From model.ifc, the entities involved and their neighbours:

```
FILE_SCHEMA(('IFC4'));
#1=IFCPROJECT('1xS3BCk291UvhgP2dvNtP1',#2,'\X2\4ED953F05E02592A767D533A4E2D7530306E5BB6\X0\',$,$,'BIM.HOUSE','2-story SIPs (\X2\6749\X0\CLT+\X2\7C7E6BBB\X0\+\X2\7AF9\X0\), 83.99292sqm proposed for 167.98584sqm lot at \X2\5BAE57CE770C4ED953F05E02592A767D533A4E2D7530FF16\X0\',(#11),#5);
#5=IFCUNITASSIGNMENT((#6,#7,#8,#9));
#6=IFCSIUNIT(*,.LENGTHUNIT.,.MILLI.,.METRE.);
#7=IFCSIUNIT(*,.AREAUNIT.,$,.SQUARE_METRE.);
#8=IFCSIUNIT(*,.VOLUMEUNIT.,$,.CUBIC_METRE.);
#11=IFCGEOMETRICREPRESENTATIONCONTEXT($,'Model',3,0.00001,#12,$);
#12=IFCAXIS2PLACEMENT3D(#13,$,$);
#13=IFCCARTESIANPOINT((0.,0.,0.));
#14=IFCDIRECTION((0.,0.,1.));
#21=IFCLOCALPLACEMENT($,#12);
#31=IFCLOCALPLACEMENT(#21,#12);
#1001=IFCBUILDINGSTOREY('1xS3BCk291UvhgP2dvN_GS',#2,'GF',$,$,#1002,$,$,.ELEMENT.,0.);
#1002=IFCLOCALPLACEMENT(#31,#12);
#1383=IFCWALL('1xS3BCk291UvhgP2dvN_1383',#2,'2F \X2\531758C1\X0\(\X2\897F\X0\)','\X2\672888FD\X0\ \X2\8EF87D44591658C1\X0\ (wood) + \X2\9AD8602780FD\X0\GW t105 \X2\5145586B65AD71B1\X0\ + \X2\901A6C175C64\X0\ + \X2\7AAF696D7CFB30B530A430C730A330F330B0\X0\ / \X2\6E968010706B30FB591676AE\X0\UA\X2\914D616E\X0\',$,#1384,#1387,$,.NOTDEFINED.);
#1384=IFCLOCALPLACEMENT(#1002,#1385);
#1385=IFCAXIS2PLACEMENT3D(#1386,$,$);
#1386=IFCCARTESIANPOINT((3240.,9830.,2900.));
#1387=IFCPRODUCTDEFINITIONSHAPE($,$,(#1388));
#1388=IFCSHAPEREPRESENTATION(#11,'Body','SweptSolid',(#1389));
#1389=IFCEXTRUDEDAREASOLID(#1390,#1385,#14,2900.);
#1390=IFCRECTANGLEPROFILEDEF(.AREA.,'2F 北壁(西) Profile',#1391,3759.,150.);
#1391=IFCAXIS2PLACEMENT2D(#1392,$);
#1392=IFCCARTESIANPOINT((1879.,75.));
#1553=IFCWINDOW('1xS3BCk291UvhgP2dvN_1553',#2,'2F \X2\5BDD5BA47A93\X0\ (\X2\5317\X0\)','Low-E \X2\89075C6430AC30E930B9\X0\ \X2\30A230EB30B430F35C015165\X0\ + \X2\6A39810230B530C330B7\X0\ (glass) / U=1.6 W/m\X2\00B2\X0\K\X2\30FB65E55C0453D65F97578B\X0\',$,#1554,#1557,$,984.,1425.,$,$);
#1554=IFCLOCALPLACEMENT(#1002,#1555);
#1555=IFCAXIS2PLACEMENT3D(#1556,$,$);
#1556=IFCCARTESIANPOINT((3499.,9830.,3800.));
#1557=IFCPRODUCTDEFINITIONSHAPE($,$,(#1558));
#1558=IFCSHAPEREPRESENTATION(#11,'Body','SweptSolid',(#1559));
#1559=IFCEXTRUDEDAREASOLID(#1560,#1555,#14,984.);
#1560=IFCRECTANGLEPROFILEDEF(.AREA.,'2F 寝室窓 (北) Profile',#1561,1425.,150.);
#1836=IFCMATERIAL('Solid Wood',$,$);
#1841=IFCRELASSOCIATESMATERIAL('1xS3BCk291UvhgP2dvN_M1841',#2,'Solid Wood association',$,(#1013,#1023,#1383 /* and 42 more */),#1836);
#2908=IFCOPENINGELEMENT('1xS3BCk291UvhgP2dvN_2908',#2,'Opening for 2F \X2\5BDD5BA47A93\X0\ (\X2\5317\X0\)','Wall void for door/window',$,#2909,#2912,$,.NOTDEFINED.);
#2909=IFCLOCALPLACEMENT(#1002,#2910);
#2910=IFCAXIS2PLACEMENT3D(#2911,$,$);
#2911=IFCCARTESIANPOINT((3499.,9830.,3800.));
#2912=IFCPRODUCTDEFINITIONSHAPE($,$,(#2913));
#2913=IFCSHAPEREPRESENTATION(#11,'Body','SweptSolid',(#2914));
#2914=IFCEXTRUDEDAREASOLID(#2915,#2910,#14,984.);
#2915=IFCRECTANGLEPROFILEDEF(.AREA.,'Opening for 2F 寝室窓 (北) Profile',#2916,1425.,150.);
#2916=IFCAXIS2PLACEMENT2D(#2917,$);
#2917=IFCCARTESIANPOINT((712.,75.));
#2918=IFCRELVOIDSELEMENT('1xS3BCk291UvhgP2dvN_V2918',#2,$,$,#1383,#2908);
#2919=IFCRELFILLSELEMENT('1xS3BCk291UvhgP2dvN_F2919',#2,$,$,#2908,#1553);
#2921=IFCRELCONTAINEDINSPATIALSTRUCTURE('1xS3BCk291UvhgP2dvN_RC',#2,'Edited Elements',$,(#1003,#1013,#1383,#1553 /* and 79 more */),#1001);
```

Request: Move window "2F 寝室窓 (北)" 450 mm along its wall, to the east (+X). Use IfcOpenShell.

```python
import ifcopenshell
import ifcopenshell.api.geometry
import ifcopenshell.util.placement
import ifcopenshell.util.unit

model = ifcopenshell.open("model.ifc")
unit_scale = ifcopenshell.util.unit.calculate_unit_scale(model)

window = model.by_id(1553)
opening = window.FillsVoids[0].RelatingOpeningElement
wall = opening.VoidsElements[0].RelatingBuildingElement

wall_matrix = ifcopenshell.util.placement.get_local_placement(wall.ObjectPlacement)
shift = wall_matrix[:3, 0] * 0.45 / unit_scale
before = ifcopenshell.util.placement.get_local_placement(window.ObjectPlacement)[:3, 3].copy()

# The window is not placed relative to its opening, so move both.
for product in (opening, window):
    matrix = ifcopenshell.util.placement.get_local_placement(product.ObjectPlacement)
    matrix[:3, 3] += shift
    ifcopenshell.api.geometry.edit_object_placement(model, product=product, matrix=matrix, is_si=False)

after = ifcopenshell.util.placement.get_local_placement(window.ObjectPlacement)[:3, 3]
print("window moved by", (after - before).round(3) + 0.0)

model.write("model_updated.ifc")
```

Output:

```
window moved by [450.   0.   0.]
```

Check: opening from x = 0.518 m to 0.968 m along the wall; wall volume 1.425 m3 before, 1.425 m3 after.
